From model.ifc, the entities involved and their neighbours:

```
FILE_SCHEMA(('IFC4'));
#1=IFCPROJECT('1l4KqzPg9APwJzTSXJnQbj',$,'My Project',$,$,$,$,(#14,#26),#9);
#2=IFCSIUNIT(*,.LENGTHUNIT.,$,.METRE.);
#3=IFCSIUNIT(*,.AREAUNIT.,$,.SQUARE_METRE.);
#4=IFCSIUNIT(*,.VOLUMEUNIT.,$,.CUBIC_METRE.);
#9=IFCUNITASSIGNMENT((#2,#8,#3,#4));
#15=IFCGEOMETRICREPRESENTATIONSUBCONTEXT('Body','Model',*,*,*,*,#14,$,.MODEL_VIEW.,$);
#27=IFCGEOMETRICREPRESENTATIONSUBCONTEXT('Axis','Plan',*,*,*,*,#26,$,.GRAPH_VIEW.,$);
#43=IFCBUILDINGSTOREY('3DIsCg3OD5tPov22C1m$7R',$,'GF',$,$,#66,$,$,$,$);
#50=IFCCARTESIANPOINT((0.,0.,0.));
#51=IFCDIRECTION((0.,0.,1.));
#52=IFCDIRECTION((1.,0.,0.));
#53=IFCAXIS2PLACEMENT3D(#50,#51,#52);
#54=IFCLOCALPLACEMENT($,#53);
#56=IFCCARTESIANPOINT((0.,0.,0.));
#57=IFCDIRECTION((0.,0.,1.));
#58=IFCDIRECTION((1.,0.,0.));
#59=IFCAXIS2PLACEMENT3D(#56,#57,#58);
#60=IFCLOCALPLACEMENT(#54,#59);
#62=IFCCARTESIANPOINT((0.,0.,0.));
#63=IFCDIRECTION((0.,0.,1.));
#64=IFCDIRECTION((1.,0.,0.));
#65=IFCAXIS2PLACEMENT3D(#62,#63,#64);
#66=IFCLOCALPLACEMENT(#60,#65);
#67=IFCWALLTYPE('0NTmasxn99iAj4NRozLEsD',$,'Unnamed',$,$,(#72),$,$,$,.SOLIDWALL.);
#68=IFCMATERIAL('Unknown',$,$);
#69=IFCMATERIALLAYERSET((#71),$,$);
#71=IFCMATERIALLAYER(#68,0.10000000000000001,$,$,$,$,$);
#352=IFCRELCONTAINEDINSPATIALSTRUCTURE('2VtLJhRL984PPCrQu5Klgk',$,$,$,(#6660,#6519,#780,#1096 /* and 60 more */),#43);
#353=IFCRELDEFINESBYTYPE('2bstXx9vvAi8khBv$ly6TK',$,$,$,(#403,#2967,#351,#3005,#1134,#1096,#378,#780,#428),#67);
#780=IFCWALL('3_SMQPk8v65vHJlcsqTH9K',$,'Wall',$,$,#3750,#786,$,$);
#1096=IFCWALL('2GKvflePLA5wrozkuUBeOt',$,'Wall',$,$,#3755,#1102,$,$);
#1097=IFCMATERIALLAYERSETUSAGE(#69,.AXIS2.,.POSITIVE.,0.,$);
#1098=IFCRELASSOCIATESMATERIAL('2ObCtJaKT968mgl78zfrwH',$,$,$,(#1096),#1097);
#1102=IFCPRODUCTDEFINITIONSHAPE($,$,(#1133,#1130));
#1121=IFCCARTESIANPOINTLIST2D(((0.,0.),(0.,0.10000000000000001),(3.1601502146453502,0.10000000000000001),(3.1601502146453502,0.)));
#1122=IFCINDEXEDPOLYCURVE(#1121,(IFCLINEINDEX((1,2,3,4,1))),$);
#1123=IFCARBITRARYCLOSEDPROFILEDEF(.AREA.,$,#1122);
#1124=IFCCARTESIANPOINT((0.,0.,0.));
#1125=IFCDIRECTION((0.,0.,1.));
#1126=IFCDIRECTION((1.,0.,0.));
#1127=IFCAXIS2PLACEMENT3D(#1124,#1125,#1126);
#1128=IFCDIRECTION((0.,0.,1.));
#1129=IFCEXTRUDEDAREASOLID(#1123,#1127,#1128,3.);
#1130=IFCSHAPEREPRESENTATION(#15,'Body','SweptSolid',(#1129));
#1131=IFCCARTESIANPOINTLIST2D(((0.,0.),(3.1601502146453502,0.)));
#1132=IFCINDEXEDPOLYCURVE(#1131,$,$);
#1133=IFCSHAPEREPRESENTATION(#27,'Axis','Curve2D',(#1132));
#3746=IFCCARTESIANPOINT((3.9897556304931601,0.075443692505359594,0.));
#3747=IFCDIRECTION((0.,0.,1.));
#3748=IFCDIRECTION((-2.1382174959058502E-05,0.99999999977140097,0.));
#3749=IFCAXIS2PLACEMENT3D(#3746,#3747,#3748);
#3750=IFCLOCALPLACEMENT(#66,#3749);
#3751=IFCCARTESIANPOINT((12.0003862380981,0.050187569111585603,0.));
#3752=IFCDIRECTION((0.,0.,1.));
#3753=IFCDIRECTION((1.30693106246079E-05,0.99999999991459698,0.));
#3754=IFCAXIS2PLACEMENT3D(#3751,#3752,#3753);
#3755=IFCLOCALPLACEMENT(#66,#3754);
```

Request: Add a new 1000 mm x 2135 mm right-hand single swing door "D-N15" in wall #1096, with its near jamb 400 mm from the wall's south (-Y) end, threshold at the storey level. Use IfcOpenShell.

```python
import numpy as np
import ifcopenshell
import ifcopenshell.api.feature
import ifcopenshell.api.geometry
import ifcopenshell.api.root
import ifcopenshell.api.spatial
import ifcopenshell.geom
import ifcopenshell.util.element
import ifcopenshell.util.placement
import ifcopenshell.util.representation
import ifcopenshell.util.shape
import ifcopenshell.util.unit

model = ifcopenshell.open("model.ifc")
unit_scale = ifcopenshell.util.unit.calculate_unit_scale(model)
settings = ifcopenshell.geom.settings()


def volume(element):
    """Net volume in cubic metres, openings subtracted."""
    shape = ifcopenshell.geom.create_shape(settings, element)
    return ifcopenshell.util.shape.get_volume(shape.geometry)


wall = model.by_id(1096)
storey = ifcopenshell.util.element.get_container(wall, ifc_class="IfcBuildingStorey")
context = ifcopenshell.util.representation.get_context(model, "Model", "Body", "MODEL_VIEW")
before = volume(wall)

width, height, from_end, sill = 1, 2.135, 0.4, 0.0  # metres

# The wall runs along its own X axis, and the end named is its -X end.
wall_shape = ifcopenshell.geom.create_shape(settings, wall)
x, y, z = ifcopenshell.util.shape.get_vertices(wall_shape.geometry).T
start = x.min() + from_end
face, thickness = float(y.min()), float(y.max() - y.min())
wall_matrix = ifcopenshell.util.placement.get_local_placement(wall.ObjectPlacement)
level = ifcopenshell.util.placement.get_local_placement(storey.ObjectPlacement)[2, 3]


def in_wall(x, y):
    """Placement at x, y metres in the wall's axes, at sill height."""
    matrix = wall_matrix.copy()
    matrix[:, 3] = wall_matrix @ np.array([x / unit_scale, y / unit_scale, 0.0, 1.0])
    matrix[2, 3] = level + sill / unit_scale
    return matrix


# Opening: a box that overshoots both wall faces by 50 mm.
opening = ifcopenshell.api.root.create_entity(model, ifc_class="IfcOpeningElement", predefined_type="OPENING")
box = ifcopenshell.api.geometry.add_wall_representation(
    model, context=context, length=width, height=height, thickness=thickness + 0.1
)
ifcopenshell.api.geometry.assign_representation(model, product=opening, representation=box)
ifcopenshell.api.geometry.edit_object_placement(model, product=opening, matrix=in_wall(start, face - 0.05), is_si=False)
ifcopenshell.api.feature.add_feature(model, feature=opening, element=wall)

door = ifcopenshell.api.root.create_entity(model, ifc_class="IfcDoor", name="D-N15", predefined_type="DOOR")
door.OverallWidth, door.OverallHeight = width / unit_scale, height / unit_scale
door.OperationType = "SINGLE_SWING_RIGHT"
body = ifcopenshell.api.geometry.add_door_representation(
    model,
    context=context,
    overall_width=door.OverallWidth,
    overall_height=door.OverallHeight,
    operation_type="SINGLE_SWING_RIGHT",
    lining_properties={"LiningDepth": thickness / unit_scale, "ThresholdDepth": thickness / unit_scale},
)
ifcopenshell.api.geometry.assign_representation(model, product=door, representation=body)
ifcopenshell.api.spatial.assign_container(model, products=[door], relating_structure=storey)
ifcopenshell.api.feature.add_filling(model, opening=opening, element=door)

# The lining spans the wall, so the door starts at the wall face.
ifcopenshell.api.geometry.edit_object_placement(model, product=door, matrix=in_wall(start, face), is_si=False)

after = volume(wall)

print(f"wall volume {before:.3f} -> {after:.3f} m3")

model.write("model_edited.ifc")
```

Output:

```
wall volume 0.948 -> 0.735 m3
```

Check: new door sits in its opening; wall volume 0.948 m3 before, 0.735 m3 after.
